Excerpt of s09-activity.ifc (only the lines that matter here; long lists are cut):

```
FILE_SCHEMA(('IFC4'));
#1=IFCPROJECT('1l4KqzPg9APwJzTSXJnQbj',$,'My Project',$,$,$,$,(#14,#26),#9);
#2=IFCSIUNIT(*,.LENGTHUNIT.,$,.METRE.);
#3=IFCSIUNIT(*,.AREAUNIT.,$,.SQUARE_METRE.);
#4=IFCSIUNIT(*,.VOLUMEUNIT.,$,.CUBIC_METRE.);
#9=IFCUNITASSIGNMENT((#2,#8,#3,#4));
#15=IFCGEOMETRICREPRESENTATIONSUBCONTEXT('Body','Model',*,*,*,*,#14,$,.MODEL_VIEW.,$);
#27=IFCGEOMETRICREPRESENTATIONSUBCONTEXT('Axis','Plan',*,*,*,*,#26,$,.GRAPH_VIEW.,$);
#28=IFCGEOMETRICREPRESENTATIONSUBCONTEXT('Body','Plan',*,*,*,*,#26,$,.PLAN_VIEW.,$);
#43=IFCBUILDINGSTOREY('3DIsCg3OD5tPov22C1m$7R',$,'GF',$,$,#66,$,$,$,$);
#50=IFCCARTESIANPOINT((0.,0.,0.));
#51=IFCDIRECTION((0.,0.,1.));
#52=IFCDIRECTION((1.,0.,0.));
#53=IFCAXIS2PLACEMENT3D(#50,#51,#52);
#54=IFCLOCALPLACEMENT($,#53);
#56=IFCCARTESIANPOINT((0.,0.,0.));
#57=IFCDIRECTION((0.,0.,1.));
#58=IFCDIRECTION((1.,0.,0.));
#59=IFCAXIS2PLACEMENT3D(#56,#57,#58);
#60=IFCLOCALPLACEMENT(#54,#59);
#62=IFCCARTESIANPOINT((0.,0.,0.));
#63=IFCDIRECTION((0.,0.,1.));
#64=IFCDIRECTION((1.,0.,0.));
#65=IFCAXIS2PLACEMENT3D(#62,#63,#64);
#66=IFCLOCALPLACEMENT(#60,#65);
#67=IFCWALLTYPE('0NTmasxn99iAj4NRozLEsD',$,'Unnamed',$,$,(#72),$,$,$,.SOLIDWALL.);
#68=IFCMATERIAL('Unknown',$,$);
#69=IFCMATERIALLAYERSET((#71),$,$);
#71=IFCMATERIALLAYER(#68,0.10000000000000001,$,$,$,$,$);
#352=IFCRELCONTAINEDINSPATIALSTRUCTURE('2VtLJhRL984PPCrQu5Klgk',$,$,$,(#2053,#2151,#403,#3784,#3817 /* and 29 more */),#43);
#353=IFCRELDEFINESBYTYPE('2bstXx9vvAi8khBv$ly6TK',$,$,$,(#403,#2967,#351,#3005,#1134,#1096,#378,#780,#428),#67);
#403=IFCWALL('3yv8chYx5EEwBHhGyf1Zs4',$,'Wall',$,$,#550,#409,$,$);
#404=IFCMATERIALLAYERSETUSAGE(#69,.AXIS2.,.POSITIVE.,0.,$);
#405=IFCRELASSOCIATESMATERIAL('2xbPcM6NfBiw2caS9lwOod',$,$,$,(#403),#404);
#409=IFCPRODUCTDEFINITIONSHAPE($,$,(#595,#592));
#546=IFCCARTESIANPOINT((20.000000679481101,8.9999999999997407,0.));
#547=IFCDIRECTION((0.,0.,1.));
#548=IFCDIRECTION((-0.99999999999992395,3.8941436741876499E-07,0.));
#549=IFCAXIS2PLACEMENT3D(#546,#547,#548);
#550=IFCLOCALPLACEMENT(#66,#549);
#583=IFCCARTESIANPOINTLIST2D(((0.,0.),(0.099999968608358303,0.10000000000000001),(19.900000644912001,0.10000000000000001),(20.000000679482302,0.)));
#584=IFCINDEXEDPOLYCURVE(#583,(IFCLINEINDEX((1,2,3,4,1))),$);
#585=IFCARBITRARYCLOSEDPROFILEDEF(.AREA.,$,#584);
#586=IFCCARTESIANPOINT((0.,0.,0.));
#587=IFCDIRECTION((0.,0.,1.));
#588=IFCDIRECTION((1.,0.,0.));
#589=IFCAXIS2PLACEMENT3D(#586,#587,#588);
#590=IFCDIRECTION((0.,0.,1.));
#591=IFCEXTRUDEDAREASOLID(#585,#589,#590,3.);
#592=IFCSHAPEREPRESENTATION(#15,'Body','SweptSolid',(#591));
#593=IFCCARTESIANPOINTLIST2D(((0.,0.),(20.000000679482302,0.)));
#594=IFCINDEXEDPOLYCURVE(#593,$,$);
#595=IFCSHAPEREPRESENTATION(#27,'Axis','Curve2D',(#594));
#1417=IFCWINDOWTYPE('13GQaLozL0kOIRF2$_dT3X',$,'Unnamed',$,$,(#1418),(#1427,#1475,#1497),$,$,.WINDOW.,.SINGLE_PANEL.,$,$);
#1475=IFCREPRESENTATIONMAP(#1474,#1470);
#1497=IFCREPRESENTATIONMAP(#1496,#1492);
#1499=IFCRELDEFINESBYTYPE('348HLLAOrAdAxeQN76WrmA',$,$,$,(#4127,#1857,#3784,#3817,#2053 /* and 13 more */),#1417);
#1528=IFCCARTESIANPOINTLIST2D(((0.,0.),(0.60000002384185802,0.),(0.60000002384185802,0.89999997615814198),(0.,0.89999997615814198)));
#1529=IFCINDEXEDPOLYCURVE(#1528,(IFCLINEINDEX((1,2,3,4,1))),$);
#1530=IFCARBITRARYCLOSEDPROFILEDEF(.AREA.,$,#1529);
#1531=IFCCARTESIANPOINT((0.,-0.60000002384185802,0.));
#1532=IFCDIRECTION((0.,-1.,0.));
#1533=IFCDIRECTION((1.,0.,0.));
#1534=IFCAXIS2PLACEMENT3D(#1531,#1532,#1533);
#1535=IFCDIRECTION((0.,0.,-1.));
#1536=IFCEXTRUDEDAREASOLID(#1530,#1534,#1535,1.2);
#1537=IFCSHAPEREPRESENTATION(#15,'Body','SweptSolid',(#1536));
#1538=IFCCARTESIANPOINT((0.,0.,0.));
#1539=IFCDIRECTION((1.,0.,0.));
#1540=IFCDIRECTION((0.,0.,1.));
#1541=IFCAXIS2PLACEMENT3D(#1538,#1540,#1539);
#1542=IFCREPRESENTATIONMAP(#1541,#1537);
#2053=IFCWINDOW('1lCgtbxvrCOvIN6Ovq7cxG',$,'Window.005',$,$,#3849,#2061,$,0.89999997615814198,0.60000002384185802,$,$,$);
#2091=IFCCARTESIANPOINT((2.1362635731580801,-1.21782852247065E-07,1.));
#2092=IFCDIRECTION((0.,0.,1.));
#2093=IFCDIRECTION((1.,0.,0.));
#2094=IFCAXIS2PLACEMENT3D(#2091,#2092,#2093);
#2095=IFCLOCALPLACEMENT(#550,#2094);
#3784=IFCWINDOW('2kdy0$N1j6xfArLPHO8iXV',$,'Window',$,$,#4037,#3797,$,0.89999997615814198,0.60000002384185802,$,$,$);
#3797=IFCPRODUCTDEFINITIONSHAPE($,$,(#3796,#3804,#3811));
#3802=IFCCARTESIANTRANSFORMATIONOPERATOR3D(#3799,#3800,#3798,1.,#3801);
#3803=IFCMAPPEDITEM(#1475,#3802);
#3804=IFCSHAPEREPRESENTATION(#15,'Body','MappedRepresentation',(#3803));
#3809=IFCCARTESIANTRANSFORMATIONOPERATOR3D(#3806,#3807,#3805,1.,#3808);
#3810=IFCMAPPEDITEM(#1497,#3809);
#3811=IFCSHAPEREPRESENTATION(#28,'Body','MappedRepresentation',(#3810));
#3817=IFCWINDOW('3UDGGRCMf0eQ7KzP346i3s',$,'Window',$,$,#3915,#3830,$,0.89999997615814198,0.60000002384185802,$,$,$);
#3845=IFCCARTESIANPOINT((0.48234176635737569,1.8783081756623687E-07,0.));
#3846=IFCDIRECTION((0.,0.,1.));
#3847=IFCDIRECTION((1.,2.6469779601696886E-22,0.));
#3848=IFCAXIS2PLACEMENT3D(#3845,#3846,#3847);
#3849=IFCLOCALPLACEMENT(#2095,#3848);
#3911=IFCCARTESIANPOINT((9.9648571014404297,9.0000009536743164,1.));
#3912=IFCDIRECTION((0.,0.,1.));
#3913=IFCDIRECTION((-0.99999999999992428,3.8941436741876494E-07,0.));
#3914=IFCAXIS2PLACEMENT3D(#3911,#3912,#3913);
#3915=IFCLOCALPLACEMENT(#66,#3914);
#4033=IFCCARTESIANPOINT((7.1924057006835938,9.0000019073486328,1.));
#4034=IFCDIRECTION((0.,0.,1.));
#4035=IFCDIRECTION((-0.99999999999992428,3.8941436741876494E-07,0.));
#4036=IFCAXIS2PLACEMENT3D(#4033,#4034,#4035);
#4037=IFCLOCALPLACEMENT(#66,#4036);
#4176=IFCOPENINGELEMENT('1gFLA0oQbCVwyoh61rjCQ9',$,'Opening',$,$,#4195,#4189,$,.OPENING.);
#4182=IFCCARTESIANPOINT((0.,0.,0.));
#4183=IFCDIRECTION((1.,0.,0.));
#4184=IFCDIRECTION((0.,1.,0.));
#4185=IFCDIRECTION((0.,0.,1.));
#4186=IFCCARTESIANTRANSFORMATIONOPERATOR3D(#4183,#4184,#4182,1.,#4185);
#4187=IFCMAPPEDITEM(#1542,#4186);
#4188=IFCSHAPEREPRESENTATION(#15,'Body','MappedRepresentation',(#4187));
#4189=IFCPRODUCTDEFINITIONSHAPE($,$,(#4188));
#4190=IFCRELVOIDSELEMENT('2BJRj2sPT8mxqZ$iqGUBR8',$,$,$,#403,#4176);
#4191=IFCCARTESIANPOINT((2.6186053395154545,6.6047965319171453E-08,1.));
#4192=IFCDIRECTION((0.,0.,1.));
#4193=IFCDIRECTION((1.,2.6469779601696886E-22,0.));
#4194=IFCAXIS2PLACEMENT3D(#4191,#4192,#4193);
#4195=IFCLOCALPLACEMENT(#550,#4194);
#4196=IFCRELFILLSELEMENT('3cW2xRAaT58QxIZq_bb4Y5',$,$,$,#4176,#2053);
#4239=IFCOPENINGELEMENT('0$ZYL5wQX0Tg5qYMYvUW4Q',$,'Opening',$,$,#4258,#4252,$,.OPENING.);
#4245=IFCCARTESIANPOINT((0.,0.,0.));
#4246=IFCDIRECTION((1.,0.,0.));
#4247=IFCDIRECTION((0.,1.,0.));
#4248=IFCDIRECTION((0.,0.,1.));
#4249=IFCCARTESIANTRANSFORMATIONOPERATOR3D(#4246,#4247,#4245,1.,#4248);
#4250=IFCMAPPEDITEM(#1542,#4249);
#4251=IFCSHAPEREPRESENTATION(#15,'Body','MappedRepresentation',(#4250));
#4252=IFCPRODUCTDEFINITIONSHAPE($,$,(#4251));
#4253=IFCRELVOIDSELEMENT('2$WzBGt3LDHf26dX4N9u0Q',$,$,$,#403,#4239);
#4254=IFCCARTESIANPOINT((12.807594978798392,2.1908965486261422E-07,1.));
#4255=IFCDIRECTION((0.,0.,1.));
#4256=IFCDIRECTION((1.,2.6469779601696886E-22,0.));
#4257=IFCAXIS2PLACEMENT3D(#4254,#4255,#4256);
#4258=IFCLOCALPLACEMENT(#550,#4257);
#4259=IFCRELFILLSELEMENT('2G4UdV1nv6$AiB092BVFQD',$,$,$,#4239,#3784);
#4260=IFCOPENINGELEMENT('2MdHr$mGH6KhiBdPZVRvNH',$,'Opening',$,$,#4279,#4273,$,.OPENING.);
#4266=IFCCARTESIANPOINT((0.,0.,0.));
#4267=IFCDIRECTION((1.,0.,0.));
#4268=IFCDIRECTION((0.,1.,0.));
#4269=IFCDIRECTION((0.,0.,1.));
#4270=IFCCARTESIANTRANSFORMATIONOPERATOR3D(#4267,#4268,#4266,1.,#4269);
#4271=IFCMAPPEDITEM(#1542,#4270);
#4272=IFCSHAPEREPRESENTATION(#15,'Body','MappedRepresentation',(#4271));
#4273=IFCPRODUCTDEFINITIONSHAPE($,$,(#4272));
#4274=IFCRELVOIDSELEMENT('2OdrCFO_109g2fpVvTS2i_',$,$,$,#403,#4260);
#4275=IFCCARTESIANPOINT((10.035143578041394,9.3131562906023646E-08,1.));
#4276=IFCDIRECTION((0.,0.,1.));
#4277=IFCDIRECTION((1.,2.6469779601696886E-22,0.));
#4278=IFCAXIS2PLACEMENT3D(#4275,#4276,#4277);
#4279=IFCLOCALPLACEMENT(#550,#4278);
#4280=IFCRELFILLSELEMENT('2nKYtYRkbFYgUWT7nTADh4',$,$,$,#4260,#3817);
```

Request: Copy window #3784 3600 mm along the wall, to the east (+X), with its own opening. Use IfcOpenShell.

```python
import ifcopenshell
import ifcopenshell.api.feature
import ifcopenshell.api.geometry
import ifcopenshell.api.root
import ifcopenshell.geom
import ifcopenshell.util.element
import ifcopenshell.util.placement
import ifcopenshell.util.shape

model = ifcopenshell.open("s09-activity.ifc")
settings = ifcopenshell.geom.settings()


def volume(element):
    """Net volume in cubic metres, openings subtracted."""
    shape = ifcopenshell.geom.create_shape(settings, element)
    return ifcopenshell.util.shape.get_volume(shape.geometry)


window = model.by_id(3784)
opening = window.FillsVoids[0].RelatingOpeningElement
wall = opening.VoidsElements[0].RelatingBuildingElement
before = volume(wall)
shift = ifcopenshell.util.placement.get_local_placement(wall.ObjectPlacement)[:3, 0] * -3.6

# copy_class copies the void relationship, type, container and properties, but no geometry.
new_opening = ifcopenshell.api.root.copy_class(model, product=opening)
new_opening.Representation = ifcopenshell.util.element.copy_deep(
    model, opening.Representation, exclude=["IfcGeometricRepresentationContext", "IfcRepresentationMap"]
)
new_window = ifcopenshell.api.root.copy_class(model, product=window)
new_window.Representation = ifcopenshell.util.element.copy_deep(
    model, window.Representation, exclude=["IfcGeometricRepresentationContext", "IfcRepresentationMap"]
)
ifcopenshell.api.feature.add_filling(model, opening=new_opening, element=new_window)

for old, new in ((opening, new_opening), (window, new_window)):
    matrix = ifcopenshell.util.placement.get_local_placement(old.ObjectPlacement)
    matrix[:3, 3] += shift
    ifcopenshell.api.geometry.edit_object_placement(model, product=new, matrix=matrix, is_si=False)

after = volume(wall)

print(f"wall volume {before:.3f} -> {after:.3f} m3")

model.write("s09-activity_v2.ifc")
```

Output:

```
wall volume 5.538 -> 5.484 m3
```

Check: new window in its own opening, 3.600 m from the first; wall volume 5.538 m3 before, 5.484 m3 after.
